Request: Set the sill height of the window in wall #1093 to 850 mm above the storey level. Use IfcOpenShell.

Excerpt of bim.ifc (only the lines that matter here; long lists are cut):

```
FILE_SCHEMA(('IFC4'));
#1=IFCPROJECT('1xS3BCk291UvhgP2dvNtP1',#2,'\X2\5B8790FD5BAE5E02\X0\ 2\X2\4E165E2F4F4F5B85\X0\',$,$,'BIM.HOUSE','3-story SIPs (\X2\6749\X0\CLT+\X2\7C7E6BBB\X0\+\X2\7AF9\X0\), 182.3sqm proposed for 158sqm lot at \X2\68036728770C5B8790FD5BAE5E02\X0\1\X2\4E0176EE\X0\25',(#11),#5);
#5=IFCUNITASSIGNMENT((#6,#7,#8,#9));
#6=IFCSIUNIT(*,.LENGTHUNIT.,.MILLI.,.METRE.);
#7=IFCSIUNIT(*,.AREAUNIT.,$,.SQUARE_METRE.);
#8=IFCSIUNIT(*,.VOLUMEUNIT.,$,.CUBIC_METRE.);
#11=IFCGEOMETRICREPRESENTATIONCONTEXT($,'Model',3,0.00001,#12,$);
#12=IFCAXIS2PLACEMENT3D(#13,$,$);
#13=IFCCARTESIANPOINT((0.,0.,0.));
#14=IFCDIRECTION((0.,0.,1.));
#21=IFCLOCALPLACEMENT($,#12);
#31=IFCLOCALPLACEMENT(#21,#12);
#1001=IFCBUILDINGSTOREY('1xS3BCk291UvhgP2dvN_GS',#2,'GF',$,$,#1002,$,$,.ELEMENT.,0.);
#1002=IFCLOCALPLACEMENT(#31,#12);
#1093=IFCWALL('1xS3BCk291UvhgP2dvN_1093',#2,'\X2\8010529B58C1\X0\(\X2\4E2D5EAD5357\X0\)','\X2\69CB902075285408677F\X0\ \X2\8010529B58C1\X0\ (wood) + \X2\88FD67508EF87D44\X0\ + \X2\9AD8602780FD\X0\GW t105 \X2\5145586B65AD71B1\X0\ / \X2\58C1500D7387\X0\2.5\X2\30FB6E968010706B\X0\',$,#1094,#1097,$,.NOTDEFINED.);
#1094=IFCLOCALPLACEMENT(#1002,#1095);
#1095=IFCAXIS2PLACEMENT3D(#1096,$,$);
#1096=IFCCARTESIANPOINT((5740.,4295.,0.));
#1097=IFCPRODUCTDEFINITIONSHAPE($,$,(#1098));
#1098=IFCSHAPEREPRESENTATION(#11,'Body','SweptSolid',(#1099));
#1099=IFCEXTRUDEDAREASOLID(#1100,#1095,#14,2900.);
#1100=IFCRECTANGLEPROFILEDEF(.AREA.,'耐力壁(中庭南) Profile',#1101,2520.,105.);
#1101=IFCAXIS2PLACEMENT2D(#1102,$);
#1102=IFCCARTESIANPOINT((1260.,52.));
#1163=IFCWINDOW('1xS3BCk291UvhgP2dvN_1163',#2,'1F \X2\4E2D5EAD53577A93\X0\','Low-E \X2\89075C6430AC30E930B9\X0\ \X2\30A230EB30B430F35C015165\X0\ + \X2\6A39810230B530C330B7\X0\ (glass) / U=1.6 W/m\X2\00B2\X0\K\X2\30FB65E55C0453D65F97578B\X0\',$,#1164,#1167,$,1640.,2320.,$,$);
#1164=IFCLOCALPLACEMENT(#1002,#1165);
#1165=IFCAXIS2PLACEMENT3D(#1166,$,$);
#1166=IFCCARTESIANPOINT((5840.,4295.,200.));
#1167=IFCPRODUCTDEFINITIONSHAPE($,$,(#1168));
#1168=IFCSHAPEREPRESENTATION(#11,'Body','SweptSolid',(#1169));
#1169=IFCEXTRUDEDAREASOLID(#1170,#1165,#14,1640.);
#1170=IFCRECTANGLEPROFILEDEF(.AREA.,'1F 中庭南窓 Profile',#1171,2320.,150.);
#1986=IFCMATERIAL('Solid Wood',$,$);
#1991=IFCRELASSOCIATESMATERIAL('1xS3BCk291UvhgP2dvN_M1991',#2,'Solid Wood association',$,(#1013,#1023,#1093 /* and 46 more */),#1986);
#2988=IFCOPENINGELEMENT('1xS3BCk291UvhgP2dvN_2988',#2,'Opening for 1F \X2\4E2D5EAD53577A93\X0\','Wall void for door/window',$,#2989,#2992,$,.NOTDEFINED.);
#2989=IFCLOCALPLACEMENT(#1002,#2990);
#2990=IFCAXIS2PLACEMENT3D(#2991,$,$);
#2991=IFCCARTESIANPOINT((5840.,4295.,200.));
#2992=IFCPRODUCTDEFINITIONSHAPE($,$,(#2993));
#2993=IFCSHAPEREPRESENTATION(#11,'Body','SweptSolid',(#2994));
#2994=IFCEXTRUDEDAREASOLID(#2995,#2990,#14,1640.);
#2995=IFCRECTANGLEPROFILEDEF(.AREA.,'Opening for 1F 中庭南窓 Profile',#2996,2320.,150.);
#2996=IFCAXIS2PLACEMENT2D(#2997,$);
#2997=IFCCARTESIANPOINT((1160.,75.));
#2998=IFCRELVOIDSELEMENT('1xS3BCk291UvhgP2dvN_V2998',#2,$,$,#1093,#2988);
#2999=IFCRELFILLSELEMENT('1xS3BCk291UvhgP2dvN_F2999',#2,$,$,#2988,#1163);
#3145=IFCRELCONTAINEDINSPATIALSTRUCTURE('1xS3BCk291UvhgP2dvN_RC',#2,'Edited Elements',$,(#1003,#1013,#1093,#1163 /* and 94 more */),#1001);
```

```python
import numpy as np
import ifcopenshell
import ifcopenshell.api.geometry
import ifcopenshell.geom
import ifcopenshell.util.element
import ifcopenshell.util.placement
import ifcopenshell.util.shape
import ifcopenshell.util.unit

model = ifcopenshell.open("bim.ifc")
unit_scale = ifcopenshell.util.unit.calculate_unit_scale(model)

window = model.by_guid("1xS3BCk291UvhgP2dvN_1163")
opening = window.FillsVoids[0].RelatingOpeningElement
storey = ifcopenshell.util.element.get_container(window, ifc_class="IfcBuildingStorey")
level = ifcopenshell.util.placement.get_local_placement(storey.ObjectPlacement)[2, 3]

# The opening's origin need not be at the sill, so measure its lowest point.
shape = ifcopenshell.geom.create_shape(ifcopenshell.geom.settings(), opening)
bottom = ifcopenshell.util.shape.get_shape_bottom_elevation(shape, shape.geometry) / unit_scale
dz = level + 850.0 - bottom

shift = np.array([0.0, 0.0, dz])
# The window is not placed relative to its opening, so move both.
for product in (opening, window):
    matrix = ifcopenshell.util.placement.get_local_placement(product.ObjectPlacement)
    matrix[:3, 3] += shift
    ifcopenshell.api.geometry.edit_object_placement(model, product=product, matrix=matrix, is_si=False)

print(f"moved by {dz * unit_scale:+.3f} m")

model.write("bim_updated.ifc")
```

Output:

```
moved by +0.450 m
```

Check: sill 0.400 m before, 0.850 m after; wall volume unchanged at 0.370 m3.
